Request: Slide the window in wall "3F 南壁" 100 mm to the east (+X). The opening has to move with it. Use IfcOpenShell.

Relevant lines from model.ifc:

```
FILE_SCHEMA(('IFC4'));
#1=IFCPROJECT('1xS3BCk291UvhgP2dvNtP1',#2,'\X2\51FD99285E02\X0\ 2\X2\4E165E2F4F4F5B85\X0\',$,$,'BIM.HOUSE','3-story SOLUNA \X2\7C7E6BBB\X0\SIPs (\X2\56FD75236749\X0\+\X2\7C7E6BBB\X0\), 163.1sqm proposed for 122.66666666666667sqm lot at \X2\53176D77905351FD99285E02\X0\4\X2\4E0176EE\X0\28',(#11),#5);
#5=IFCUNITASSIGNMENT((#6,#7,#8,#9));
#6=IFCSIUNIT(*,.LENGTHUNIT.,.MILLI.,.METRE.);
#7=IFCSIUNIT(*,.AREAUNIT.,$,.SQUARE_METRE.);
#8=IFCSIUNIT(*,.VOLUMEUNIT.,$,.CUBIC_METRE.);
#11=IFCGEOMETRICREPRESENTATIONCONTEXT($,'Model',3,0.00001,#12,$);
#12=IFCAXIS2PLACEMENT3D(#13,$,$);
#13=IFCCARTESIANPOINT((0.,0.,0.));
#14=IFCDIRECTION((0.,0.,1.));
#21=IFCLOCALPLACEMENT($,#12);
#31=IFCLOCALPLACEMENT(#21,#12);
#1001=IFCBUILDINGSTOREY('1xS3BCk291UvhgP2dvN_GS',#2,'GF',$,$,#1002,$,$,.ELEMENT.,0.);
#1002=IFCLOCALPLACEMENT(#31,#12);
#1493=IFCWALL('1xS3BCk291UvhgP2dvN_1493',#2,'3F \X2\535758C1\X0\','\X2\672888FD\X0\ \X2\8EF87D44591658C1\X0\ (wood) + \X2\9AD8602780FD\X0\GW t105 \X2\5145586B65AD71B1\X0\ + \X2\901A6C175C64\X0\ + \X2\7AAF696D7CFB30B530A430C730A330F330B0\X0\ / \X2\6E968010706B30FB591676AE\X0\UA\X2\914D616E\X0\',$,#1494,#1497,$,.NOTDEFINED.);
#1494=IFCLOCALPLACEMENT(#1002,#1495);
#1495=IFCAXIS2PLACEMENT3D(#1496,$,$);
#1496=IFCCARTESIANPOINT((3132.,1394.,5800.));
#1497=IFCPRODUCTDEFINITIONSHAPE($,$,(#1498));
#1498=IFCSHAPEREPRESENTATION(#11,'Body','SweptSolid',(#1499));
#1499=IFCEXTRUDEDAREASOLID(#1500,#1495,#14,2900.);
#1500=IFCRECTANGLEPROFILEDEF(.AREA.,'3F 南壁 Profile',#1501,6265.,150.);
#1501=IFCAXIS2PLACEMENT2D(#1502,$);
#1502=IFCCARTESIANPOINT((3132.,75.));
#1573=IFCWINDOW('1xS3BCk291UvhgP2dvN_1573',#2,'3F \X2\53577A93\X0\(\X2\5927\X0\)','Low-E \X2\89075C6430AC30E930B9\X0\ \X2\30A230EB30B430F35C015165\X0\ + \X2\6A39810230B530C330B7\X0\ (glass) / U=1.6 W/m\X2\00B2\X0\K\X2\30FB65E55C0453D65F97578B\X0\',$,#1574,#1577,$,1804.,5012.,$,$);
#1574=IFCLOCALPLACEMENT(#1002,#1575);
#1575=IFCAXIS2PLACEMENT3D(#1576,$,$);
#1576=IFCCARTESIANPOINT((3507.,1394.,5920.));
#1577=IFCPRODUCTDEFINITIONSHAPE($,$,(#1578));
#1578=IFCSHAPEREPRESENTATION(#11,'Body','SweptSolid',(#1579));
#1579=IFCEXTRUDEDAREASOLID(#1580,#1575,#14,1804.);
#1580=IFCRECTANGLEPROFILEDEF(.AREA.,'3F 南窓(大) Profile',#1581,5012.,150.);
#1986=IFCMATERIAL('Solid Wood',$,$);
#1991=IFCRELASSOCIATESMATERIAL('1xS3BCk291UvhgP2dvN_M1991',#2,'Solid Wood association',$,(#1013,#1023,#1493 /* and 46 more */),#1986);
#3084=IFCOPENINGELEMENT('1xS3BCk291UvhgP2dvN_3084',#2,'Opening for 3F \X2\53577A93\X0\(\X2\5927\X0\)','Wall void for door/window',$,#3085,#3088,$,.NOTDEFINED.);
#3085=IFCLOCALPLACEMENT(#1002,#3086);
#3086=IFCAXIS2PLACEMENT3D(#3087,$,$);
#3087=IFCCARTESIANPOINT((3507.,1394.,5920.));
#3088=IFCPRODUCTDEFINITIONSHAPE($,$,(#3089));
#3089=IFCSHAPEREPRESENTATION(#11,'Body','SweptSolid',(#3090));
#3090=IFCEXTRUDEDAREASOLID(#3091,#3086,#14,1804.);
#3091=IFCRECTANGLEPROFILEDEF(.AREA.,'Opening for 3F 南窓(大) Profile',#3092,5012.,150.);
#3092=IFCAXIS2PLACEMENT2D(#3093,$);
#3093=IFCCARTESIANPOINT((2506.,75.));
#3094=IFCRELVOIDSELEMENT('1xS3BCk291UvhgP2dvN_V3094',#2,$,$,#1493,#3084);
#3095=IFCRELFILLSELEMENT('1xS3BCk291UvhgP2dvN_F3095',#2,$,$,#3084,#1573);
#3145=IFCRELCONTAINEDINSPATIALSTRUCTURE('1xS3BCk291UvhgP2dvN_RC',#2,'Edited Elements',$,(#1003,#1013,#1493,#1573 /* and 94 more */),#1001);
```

```python
import ifcopenshell
import ifcopenshell.api.geometry
import ifcopenshell.util.placement

model = ifcopenshell.open("model.ifc")

window = model.by_guid("1xS3BCk291UvhgP2dvN_1573")
opening = window.FillsVoids[0].RelatingOpeningElement
wall = opening.VoidsElements[0].RelatingBuildingElement

wall_matrix = ifcopenshell.util.placement.get_local_placement(wall.ObjectPlacement)
shift = wall_matrix[:3, 0] * 100.0
before = ifcopenshell.util.placement.get_local_placement(window.ObjectPlacement)[:3, 3].copy()

# The window is not placed relative to its opening, so move both.
for product in (opening, window):
    matrix = ifcopenshell.util.placement.get_local_placement(product.ObjectPlacement)
    matrix[:3, 3] += shift
    ifcopenshell.api.geometry.edit_object_placement(model, product=product, matrix=matrix, is_si=False)

after = ifcopenshell.util.placement.get_local_placement(window.ObjectPlacement)[:3, 3]
print("window moved by", (after - before).round(3) + 0.0)

model.write("model_updated.ifc")
```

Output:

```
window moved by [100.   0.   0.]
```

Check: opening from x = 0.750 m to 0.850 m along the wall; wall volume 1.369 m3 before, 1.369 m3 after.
